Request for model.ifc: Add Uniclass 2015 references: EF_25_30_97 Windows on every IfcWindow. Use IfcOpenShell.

First a look at what the model holds.

```python
import ifcopenshell

model = ifcopenshell.open("model.ifc")
print(model.schema)
print("classifications:", [c.Name for c in model.by_type("IfcClassification")])
for ifc_class in ("IfcDoor", "IfcRoof", "IfcStair", "IfcWall", "IfcWindow"):
    print(ifc_class, len(model.by_type(ifc_class)))
```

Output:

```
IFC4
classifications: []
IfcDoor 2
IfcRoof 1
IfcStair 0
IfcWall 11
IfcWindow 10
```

```python
import ifcopenshell
import ifcopenshell.api.classification

model = ifcopenshell.open("model.ifc")

system = ifcopenshell.api.classification.add_classification(model, classification="Uniclass 2015")

codes = {
    "IfcWindow": ("EF_25_30_97", "Windows"),
}
for ifc_class, (code, name) in codes.items():
    products = model.by_type(ifc_class)
    ifcopenshell.api.classification.add_reference(
        model, products=products, classification=system, identification=code, name=name
    )
    print(code, len(products))

model.write("model_v2.ifc")
```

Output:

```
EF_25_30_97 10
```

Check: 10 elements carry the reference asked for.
